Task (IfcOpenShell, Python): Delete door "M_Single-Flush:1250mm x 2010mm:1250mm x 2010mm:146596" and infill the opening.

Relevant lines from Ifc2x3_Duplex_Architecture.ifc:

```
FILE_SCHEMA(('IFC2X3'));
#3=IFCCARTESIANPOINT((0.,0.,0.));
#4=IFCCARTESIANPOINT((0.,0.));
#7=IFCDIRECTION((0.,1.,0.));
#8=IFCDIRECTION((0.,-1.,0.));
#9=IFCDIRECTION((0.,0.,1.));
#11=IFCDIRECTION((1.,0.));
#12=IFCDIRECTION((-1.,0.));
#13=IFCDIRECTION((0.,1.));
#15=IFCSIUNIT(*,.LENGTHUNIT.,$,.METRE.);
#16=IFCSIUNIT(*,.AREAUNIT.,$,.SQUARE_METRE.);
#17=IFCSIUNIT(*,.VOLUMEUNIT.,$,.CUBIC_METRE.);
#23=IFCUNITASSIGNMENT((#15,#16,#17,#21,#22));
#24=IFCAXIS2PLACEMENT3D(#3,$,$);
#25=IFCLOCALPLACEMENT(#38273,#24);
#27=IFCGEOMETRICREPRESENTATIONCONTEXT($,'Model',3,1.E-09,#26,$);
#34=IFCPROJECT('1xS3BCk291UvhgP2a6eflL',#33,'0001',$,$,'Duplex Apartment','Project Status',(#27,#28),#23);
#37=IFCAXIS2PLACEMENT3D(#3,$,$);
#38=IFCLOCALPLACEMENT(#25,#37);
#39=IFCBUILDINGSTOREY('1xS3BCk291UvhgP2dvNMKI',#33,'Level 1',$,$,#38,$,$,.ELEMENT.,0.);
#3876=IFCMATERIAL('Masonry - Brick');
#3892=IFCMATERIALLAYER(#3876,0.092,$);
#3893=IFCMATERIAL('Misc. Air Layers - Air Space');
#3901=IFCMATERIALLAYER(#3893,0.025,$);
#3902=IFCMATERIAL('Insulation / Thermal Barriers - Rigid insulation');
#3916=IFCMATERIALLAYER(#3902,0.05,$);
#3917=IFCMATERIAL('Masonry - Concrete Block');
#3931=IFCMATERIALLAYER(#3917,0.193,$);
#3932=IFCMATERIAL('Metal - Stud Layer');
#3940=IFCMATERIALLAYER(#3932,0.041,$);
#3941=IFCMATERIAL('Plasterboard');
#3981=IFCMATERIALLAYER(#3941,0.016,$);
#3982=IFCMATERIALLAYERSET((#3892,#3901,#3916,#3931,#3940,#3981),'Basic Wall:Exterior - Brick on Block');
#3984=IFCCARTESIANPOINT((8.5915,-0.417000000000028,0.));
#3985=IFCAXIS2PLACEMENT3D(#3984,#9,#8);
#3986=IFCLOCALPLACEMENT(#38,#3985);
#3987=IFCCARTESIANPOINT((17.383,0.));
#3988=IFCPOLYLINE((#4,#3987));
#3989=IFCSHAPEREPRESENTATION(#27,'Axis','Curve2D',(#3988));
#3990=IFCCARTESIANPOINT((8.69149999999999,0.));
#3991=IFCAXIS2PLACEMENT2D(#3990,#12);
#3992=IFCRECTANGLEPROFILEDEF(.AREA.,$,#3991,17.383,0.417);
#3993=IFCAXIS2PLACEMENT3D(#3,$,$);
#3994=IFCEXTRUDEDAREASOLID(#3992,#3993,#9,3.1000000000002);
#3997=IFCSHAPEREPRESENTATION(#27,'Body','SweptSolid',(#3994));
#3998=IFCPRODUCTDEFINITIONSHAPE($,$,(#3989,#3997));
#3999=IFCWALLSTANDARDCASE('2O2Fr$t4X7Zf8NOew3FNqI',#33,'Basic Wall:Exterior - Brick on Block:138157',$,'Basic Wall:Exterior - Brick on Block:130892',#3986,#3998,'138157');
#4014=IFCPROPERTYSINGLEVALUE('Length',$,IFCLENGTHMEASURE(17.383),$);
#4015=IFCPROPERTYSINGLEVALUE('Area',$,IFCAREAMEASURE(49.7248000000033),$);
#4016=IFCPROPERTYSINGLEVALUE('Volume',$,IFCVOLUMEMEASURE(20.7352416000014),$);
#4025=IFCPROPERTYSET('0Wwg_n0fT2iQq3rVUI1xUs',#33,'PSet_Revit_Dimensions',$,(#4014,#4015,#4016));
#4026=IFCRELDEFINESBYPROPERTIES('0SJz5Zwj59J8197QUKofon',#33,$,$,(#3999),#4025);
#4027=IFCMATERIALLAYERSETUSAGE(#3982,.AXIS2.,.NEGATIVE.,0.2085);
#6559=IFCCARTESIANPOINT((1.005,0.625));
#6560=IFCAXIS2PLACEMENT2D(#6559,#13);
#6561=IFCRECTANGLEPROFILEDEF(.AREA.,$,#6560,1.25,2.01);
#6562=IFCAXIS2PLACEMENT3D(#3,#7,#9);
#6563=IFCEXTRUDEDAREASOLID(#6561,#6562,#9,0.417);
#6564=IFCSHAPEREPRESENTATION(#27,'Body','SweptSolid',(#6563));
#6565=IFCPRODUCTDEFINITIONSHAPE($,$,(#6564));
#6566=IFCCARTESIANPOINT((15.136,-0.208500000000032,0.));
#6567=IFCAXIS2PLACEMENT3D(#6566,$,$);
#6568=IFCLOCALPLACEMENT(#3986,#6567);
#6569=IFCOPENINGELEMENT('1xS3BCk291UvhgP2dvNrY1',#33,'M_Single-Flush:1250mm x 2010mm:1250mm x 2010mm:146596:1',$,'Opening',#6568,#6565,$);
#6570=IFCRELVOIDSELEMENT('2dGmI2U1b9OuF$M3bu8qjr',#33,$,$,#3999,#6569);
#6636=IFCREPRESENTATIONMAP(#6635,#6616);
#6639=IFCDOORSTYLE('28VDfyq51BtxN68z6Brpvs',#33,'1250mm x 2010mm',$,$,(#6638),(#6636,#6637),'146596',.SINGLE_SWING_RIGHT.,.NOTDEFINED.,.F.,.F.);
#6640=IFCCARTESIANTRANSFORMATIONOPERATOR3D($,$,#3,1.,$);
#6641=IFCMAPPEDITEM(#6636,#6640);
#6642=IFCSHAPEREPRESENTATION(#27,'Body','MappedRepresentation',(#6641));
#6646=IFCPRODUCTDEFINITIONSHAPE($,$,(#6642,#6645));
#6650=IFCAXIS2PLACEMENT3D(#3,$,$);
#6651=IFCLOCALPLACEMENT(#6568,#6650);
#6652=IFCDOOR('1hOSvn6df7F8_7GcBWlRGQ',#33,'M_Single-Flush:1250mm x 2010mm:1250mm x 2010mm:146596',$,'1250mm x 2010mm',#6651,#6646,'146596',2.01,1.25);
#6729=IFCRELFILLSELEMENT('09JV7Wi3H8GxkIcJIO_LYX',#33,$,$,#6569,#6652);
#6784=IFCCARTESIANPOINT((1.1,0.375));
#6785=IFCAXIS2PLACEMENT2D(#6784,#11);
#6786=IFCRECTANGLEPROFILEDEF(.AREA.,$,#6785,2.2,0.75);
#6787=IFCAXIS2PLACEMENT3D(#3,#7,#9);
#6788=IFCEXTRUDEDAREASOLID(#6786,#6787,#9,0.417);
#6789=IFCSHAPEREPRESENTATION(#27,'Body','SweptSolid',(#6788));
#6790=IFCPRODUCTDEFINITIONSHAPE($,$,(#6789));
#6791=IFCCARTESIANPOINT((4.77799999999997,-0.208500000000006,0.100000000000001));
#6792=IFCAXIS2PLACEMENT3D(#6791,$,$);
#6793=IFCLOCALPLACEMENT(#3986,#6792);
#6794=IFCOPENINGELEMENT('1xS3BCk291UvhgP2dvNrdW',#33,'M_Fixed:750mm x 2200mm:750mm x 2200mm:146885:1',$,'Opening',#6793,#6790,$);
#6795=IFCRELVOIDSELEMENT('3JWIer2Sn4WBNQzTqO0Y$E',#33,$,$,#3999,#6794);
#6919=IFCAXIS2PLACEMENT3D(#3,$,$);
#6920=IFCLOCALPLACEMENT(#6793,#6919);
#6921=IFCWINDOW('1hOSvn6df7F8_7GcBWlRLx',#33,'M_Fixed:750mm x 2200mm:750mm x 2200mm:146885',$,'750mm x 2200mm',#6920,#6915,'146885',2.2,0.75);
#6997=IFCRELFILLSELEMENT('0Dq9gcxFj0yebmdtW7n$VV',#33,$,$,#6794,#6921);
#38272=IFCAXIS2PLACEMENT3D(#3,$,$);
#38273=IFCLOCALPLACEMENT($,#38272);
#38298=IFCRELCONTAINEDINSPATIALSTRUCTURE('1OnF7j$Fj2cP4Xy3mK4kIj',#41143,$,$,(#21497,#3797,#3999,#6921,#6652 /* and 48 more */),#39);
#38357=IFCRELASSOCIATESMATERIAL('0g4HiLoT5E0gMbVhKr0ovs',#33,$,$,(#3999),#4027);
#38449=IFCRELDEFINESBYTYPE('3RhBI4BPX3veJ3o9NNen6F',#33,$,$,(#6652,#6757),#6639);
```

```python
import ifcopenshell
import ifcopenshell.api.feature
import ifcopenshell.api.pset
import ifcopenshell.api.root
import ifcopenshell.geom
import ifcopenshell.util.element
import ifcopenshell.util.shape
import ifcopenshell.util.unit

model = ifcopenshell.open("Ifc2x3_Duplex_Architecture.ifc")
area_scale = ifcopenshell.util.unit.calculate_unit_scale(model, "AREAUNIT")
volume_scale = ifcopenshell.util.unit.calculate_unit_scale(model, "VOLUMEUNIT")
settings = ifcopenshell.geom.settings()


def volume(element):
    """Net volume in cubic metres, openings subtracted."""
    shape = ifcopenshell.geom.create_shape(settings, element)
    return ifcopenshell.util.shape.get_volume(shape.geometry)


door = model.by_guid("1hOSvn6df7F8_7GcBWlRGQ")
opening = door.FillsVoids[0].RelatingOpeningElement
wall = opening.VoidsElements[0].RelatingBuildingElement
before = volume(wall)

ifcopenshell.api.root.remove_product(model, product=door)
ifcopenshell.api.feature.remove_feature(model, feature=opening)

after = volume(wall)
thickness = 0.417  # wall thickness in metres

# Update the wall's stored quantities.
pset = model.by_id(ifcopenshell.util.element.get_pset(wall, "PSet_Revit_Dimensions", should_inherit=False)["id"])
ifcopenshell.api.pset.edit_pset(model, pset=pset, properties={
    "Area": model.create_entity("IfcAreaMeasure", after / thickness / area_scale),
    "Volume": model.create_entity("IfcVolumeMeasure", after / volume_scale),
})

print(f"wall volume {before:.3f} -> {after:.3f} m3")

model.write("Ifc2x3_Duplex_Architecture-out.ifc")
```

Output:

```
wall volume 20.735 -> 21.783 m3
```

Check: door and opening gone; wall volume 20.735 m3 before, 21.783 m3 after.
